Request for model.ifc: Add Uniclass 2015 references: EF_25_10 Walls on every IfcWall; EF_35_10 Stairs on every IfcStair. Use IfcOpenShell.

First a look at what the model holds.

```python
import ifcopenshell

model = ifcopenshell.open("model.ifc")
print(model.schema)
print("classifications:", [c.Name for c in model.by_type("IfcClassification")])
for ifc_class in ("IfcDoor", "IfcRoof", "IfcStair", "IfcWall", "IfcWindow"):
    print(ifc_class, len(model.by_type(ifc_class)))
```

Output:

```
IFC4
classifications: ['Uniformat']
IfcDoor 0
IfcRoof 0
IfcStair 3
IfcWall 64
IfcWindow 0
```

```python
import ifcopenshell
import ifcopenshell.api.classification

model = ifcopenshell.open("model.ifc")

system = ifcopenshell.api.classification.add_classification(model, classification="Uniclass 2015")

codes = {
    "IfcWall": ("EF_25_10", "Walls"),
    "IfcStair": ("EF_35_10", "Stairs"),
}
for ifc_class, (code, name) in codes.items():
    products = model.by_type(ifc_class)
    ifcopenshell.api.classification.add_reference(
        model, products=products, classification=system, identification=code, name=name
    )
    print(code, len(products))

model.write("model_edited.ifc")
```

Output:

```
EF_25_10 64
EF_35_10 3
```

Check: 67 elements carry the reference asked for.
